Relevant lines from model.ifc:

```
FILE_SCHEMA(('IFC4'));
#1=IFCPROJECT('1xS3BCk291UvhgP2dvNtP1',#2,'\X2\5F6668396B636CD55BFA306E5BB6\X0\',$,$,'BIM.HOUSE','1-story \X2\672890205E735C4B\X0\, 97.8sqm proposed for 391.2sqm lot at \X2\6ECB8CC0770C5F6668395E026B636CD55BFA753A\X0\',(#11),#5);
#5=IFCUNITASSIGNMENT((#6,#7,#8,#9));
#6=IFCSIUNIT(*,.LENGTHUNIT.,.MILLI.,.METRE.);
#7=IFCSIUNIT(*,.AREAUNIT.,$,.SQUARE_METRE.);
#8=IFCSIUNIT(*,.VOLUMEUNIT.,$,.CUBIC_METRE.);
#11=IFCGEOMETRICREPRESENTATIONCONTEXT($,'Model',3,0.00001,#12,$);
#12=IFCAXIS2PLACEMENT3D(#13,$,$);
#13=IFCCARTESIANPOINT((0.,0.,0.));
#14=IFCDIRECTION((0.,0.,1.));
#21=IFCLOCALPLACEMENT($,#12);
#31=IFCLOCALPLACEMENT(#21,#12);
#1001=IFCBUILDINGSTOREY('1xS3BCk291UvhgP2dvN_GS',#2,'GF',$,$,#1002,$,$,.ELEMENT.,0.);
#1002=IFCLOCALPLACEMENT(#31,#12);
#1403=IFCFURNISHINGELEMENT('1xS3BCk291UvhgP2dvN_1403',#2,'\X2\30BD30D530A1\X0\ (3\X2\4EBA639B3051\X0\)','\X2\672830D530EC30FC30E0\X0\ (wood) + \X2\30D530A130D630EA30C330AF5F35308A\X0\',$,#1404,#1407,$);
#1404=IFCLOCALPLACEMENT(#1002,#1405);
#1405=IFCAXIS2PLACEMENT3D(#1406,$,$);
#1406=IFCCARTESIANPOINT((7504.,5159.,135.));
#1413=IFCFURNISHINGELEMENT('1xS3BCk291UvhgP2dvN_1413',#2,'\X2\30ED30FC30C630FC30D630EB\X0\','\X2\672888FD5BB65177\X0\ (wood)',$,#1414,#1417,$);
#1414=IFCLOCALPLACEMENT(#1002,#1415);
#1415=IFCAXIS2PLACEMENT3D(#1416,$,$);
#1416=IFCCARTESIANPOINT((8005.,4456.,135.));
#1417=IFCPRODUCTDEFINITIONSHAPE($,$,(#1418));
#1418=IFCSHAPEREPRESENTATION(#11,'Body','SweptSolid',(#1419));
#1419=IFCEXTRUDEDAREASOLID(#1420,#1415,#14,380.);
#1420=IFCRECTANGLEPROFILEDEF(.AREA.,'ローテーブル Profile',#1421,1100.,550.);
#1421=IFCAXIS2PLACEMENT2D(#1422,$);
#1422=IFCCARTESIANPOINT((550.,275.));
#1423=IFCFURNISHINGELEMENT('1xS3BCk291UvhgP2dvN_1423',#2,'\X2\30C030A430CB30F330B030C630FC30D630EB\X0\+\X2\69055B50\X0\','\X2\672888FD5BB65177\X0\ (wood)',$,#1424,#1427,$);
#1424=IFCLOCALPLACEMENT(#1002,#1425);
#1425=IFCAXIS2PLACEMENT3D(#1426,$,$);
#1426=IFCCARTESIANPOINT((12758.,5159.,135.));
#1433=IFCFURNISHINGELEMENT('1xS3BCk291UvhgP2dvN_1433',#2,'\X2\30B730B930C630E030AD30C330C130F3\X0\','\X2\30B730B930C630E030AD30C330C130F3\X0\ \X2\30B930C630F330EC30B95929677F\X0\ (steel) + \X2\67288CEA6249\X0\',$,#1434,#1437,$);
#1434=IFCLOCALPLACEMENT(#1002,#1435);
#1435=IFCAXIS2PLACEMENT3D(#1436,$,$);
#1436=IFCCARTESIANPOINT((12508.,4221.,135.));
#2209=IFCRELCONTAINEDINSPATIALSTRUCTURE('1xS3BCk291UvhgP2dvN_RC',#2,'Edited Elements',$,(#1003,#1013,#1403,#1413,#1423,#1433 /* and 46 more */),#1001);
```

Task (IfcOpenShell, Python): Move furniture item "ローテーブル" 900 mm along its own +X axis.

```python
import ifcopenshell
import ifcopenshell.api.geometry
import ifcopenshell.util.placement
import ifcopenshell.util.unit

model = ifcopenshell.open("model.ifc")
unit_scale = ifcopenshell.util.unit.calculate_unit_scale(model)

item = model.by_id(1413)
matrix = ifcopenshell.util.placement.get_local_placement(item.ObjectPlacement)
matrix[:3, 3] += matrix[:3, 0] * 0.9 / unit_scale
ifcopenshell.api.geometry.edit_object_placement(model, product=item, matrix=matrix, is_si=False)

print(ifcopenshell.util.placement.get_local_placement(item.ObjectPlacement).round(3) + 0.0)

model.write("model_rev.ifc")
```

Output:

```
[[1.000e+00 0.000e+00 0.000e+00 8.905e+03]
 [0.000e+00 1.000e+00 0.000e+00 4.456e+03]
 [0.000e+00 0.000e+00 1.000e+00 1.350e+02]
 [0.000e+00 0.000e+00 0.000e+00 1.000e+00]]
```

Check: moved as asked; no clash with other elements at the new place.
